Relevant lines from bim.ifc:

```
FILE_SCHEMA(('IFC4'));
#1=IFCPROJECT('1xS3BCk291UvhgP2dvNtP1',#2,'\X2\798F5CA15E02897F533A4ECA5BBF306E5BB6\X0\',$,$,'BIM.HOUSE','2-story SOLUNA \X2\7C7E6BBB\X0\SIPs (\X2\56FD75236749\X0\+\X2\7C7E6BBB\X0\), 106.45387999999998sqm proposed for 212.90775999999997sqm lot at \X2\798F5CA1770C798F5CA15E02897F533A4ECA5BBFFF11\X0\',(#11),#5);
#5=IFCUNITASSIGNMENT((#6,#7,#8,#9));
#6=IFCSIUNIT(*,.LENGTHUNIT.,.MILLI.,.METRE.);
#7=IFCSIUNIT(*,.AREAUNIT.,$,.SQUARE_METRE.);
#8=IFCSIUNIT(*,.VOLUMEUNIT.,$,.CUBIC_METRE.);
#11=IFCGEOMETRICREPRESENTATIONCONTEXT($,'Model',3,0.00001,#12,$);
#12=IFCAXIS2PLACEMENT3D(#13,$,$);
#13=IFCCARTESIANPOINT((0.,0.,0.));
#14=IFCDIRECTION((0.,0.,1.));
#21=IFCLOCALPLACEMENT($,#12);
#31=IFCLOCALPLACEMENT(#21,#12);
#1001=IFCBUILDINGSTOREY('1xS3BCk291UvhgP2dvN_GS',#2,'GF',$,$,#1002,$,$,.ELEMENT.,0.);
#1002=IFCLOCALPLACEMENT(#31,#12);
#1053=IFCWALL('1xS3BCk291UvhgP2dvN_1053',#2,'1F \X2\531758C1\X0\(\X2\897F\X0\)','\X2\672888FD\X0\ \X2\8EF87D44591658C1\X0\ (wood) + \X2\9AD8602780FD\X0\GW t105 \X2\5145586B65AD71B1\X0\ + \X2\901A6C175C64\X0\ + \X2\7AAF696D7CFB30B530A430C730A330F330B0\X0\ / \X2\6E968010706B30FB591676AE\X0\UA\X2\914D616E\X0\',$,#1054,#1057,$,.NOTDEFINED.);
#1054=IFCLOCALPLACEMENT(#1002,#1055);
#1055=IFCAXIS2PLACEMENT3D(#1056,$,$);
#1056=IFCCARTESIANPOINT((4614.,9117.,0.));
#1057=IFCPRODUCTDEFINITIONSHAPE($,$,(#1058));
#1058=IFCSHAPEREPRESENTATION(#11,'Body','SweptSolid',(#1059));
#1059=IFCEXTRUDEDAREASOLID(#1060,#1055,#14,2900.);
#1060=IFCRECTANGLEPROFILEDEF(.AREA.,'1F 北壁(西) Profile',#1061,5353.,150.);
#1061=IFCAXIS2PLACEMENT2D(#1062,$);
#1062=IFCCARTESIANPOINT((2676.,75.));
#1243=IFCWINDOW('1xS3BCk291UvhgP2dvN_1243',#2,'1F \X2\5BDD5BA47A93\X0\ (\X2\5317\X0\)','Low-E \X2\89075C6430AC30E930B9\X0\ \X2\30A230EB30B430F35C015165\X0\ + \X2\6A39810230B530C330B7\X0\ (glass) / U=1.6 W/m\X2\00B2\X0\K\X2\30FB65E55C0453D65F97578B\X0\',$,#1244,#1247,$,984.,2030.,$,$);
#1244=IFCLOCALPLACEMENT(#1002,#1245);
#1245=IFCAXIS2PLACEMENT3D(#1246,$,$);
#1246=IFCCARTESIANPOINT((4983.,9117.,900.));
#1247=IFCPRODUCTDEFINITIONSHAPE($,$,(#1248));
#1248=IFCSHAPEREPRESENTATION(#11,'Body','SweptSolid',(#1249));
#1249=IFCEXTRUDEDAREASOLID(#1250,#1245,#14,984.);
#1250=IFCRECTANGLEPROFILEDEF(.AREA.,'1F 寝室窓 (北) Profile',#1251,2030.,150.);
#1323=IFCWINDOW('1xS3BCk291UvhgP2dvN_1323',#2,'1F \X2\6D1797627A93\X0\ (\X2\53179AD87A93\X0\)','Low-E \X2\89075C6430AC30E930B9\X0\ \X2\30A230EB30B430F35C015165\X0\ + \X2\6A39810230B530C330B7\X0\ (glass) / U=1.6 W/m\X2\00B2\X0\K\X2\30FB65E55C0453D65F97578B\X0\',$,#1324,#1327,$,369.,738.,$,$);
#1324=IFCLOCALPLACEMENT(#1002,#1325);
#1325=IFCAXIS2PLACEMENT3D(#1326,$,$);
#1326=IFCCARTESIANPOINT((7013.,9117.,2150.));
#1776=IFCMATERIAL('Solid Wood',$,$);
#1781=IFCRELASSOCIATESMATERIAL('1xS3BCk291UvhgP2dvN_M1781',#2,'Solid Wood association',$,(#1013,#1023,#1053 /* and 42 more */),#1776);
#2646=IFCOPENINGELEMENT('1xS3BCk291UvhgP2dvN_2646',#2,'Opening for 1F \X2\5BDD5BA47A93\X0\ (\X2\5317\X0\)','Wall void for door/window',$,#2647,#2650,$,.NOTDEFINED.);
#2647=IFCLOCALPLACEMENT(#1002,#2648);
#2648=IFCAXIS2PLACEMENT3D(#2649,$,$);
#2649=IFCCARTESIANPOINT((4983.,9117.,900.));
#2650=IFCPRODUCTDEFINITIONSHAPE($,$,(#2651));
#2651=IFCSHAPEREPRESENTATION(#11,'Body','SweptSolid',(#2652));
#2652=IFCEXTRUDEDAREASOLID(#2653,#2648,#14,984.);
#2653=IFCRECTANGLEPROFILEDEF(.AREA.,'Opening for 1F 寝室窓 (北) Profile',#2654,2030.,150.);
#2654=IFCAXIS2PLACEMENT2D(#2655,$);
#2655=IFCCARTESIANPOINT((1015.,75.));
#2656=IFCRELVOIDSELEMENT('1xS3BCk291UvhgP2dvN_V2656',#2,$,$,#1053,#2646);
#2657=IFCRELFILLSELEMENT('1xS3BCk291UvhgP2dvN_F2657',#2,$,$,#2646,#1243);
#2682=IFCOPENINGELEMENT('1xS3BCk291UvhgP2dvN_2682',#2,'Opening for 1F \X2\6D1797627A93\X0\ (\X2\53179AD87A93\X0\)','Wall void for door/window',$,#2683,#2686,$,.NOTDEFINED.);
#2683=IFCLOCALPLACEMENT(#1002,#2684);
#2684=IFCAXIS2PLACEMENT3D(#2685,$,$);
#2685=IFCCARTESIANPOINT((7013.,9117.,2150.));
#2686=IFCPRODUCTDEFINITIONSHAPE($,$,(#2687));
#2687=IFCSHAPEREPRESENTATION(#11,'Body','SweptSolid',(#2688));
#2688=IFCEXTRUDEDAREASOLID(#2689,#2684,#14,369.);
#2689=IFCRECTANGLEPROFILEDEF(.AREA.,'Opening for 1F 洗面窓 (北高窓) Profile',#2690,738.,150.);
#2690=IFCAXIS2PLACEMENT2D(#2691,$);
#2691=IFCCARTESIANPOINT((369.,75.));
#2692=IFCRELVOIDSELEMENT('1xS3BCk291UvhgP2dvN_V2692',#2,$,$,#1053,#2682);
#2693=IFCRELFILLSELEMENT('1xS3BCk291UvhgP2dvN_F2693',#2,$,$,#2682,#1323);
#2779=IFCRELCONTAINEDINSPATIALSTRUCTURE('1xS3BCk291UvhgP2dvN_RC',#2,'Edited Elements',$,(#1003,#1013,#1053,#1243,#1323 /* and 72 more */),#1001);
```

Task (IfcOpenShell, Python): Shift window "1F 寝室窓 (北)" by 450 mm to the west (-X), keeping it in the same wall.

```python
import ifcopenshell
import ifcopenshell.api.geometry
import ifcopenshell.util.placement
import ifcopenshell.util.unit

model = ifcopenshell.open("bim.ifc")
unit_scale = ifcopenshell.util.unit.calculate_unit_scale(model)

window = model.by_id(1243)
opening = window.FillsVoids[0].RelatingOpeningElement
wall = opening.VoidsElements[0].RelatingBuildingElement

wall_matrix = ifcopenshell.util.placement.get_local_placement(wall.ObjectPlacement)
shift = wall_matrix[:3, 0] * -0.45 / unit_scale
before = ifcopenshell.util.placement.get_local_placement(window.ObjectPlacement)[:3, 3].copy()

# The window is not placed relative to its opening, so move both.
for product in (opening, window):
    matrix = ifcopenshell.util.placement.get_local_placement(product.ObjectPlacement)
    matrix[:3, 3] += shift
    ifcopenshell.api.geometry.edit_object_placement(model, product=product, matrix=matrix, is_si=False)

after = ifcopenshell.util.placement.get_local_placement(window.ObjectPlacement)[:3, 3]
print("window moved by", (after - before).round(3) + 0.0)

model.write("bim_edited.ifc")
```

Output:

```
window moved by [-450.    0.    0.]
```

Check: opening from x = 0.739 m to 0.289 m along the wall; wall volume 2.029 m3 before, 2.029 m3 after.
